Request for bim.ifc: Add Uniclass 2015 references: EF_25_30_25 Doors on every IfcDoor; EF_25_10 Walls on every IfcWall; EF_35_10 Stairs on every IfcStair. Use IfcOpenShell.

First a look at what the model holds.

```python
import ifcopenshell

model = ifcopenshell.open("bim.ifc")
print(model.schema)
print("classifications:", [c.Name for c in model.by_type("IfcClassification")])
for ifc_class in ("IfcDoor", "IfcRoof", "IfcStair", "IfcWall", "IfcWindow"):
    print(ifc_class, len(model.by_type(ifc_class)))
```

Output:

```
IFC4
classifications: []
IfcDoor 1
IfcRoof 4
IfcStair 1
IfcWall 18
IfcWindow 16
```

```python
import ifcopenshell
import ifcopenshell.api.classification

model = ifcopenshell.open("bim.ifc")

system = ifcopenshell.api.classification.add_classification(model, classification="Uniclass 2015")

codes = {
    "IfcDoor": ("EF_25_30_25", "Doors"),
    "IfcWall": ("EF_25_10", "Walls"),
    "IfcStair": ("EF_35_10", "Stairs"),
}
for ifc_class, (code, name) in codes.items():
    products = model.by_type(ifc_class)
    ifcopenshell.api.classification.add_reference(
        model, products=products, classification=system, identification=code, name=name
    )
    print(code, len(products))

model.write("bim-out.ifc")
```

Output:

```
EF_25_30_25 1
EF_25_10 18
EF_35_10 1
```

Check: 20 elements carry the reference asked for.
